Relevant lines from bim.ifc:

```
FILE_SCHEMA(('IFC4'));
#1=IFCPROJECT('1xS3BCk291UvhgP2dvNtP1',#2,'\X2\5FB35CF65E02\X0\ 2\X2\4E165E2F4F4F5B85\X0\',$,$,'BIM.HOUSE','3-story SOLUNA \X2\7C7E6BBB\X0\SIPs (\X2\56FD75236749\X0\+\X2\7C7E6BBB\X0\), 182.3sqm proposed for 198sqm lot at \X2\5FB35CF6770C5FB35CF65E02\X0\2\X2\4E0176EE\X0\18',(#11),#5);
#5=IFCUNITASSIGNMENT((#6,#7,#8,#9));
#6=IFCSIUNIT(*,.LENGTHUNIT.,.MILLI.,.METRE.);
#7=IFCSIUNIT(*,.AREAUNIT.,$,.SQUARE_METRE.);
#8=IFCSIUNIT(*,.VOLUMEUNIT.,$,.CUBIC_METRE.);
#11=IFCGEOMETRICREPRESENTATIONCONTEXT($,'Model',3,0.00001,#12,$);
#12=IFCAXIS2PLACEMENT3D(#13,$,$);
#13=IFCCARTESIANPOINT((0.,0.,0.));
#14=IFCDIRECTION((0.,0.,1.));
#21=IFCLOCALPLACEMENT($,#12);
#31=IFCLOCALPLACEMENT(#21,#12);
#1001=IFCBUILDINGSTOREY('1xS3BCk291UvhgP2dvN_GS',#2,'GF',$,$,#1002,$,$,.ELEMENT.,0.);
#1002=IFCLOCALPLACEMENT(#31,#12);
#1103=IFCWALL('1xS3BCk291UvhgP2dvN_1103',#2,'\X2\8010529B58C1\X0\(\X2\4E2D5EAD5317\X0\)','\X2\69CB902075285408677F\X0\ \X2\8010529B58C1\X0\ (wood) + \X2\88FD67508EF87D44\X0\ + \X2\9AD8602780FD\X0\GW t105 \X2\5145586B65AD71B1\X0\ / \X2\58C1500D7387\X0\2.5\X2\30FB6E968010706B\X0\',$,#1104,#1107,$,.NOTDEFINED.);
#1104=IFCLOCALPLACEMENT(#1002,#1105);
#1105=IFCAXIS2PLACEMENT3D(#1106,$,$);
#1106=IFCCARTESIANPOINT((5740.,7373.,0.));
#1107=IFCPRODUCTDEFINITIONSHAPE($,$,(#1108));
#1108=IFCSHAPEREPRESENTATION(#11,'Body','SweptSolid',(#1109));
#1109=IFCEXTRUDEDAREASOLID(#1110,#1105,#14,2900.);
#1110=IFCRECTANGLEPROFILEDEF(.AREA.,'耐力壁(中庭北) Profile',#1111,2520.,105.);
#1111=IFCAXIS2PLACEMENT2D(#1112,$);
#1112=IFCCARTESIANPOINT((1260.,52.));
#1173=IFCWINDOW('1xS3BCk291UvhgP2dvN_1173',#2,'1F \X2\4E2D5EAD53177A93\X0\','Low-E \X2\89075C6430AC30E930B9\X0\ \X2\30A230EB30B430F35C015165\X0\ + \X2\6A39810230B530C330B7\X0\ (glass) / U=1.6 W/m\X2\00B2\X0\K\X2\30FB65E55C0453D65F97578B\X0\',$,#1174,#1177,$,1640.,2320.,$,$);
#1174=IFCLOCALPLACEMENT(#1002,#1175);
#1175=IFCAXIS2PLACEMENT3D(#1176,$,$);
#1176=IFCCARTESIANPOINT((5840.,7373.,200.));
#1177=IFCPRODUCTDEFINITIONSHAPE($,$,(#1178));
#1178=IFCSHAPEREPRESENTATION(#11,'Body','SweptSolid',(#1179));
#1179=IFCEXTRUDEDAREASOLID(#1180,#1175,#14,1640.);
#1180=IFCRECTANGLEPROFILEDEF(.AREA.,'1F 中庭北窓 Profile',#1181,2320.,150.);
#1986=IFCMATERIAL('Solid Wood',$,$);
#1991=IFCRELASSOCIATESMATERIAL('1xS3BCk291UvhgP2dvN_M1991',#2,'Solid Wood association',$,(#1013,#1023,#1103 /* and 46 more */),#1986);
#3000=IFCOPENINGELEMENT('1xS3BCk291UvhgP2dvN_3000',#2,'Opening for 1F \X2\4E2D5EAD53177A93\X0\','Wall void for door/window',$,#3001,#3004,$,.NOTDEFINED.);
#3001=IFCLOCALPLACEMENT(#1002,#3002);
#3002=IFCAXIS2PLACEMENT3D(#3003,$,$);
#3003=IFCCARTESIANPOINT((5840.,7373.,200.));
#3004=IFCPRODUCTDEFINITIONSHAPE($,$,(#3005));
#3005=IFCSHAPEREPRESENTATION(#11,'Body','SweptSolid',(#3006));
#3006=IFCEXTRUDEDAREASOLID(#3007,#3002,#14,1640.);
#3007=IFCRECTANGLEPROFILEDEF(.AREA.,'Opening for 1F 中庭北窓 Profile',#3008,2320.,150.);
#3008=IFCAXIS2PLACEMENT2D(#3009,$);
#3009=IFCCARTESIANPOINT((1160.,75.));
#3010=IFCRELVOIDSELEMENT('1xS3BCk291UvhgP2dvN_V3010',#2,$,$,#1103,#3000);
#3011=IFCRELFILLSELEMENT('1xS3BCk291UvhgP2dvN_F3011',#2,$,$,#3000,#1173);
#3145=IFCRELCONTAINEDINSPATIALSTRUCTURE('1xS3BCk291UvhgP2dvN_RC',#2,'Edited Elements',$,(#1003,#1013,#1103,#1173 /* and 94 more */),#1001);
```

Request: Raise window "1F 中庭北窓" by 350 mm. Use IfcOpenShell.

```python
import numpy as np
import ifcopenshell
import ifcopenshell.api.geometry
import ifcopenshell.util.placement
import ifcopenshell.util.unit

model = ifcopenshell.open("bim.ifc")
unit_scale = ifcopenshell.util.unit.calculate_unit_scale(model)

window = model.by_id(1173)
opening = window.FillsVoids[0].RelatingOpeningElement
dz = 0.35 / unit_scale

shift = np.array([0.0, 0.0, dz])
# The window is not placed relative to its opening, so move both.
for product in (opening, window):
    matrix = ifcopenshell.util.placement.get_local_placement(product.ObjectPlacement)
    matrix[:3, 3] += shift
    ifcopenshell.api.geometry.edit_object_placement(model, product=product, matrix=matrix, is_si=False)

print(f"moved by {dz * unit_scale:+.3f} m")

model.write("bim_rev.ifc")
```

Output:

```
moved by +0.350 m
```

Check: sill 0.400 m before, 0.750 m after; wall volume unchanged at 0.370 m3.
